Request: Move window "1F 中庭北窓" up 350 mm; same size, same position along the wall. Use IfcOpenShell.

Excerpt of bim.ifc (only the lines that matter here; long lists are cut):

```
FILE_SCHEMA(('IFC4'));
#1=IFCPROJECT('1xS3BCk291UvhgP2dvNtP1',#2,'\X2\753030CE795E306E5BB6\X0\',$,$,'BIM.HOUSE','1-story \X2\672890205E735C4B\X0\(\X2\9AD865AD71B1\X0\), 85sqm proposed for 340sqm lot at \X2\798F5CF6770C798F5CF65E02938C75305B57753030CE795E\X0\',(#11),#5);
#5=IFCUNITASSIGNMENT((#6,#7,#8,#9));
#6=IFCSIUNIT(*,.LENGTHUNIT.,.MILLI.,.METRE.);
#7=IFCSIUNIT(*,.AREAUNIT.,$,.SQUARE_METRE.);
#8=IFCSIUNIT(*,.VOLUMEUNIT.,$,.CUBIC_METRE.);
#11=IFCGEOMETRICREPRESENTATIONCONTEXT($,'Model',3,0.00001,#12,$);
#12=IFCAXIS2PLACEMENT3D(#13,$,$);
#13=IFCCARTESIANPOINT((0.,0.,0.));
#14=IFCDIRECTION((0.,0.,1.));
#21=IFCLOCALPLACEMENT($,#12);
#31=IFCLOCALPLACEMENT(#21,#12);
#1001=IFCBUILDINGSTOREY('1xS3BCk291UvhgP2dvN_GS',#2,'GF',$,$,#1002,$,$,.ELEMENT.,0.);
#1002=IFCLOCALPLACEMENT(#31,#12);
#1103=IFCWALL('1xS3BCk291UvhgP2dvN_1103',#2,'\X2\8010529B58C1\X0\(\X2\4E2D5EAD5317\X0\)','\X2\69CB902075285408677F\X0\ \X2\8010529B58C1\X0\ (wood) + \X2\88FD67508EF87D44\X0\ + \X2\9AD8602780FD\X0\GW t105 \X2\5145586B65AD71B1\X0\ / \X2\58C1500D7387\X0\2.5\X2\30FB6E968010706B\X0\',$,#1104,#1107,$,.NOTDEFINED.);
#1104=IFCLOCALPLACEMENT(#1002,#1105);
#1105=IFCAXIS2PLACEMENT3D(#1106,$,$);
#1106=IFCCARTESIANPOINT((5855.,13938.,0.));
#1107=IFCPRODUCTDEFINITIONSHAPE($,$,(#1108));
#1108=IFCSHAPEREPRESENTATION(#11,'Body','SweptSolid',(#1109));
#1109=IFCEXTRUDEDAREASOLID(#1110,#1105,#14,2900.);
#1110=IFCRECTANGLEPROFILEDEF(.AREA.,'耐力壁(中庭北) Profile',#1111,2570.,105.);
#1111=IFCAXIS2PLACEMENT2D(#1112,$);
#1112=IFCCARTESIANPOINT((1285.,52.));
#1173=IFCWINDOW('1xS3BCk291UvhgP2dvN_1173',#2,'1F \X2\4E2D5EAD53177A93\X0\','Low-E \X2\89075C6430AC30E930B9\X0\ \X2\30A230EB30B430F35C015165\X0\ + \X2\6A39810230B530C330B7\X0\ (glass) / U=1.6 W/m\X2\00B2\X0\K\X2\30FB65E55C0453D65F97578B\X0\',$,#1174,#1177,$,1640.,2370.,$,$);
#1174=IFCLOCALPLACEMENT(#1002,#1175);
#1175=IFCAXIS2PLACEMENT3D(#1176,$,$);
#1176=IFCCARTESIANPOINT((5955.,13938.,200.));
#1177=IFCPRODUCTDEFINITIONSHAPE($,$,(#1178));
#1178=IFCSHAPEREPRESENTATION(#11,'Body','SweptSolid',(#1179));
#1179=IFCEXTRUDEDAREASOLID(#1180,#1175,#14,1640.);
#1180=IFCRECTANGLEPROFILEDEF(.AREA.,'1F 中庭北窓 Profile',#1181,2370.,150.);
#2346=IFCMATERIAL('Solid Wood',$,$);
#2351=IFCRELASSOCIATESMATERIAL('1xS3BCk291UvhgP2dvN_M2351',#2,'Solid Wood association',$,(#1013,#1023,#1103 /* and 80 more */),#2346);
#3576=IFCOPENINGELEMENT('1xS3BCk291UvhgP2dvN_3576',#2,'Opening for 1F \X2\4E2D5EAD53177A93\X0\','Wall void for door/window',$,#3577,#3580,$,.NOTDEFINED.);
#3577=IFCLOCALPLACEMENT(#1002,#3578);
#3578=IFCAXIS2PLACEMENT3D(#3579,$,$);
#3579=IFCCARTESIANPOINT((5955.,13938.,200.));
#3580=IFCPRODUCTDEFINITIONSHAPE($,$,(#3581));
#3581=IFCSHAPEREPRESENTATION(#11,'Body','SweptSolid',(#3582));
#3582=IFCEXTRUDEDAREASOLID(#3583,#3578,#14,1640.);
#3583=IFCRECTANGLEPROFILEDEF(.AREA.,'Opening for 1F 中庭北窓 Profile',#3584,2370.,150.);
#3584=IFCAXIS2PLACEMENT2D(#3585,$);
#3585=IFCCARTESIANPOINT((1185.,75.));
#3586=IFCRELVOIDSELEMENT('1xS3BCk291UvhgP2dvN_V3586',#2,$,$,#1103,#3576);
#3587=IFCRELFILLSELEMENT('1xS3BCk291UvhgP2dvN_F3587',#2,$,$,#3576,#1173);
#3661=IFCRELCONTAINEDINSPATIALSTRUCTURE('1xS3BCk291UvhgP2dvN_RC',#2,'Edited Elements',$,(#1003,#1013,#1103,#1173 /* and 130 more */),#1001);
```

```python
import numpy as np
import ifcopenshell
import ifcopenshell.api.geometry
import ifcopenshell.util.placement
import ifcopenshell.util.unit

model = ifcopenshell.open("bim.ifc")
unit_scale = ifcopenshell.util.unit.calculate_unit_scale(model)

window = model.by_guid("1xS3BCk291UvhgP2dvN_1173")
opening = window.FillsVoids[0].RelatingOpeningElement
dz = 0.35 / unit_scale

shift = np.array([0.0, 0.0, dz])
# The window is not placed relative to its opening, so move both.
for product in (opening, window):
    matrix = ifcopenshell.util.placement.get_local_placement(product.ObjectPlacement)
    matrix[:3, 3] += shift
    ifcopenshell.api.geometry.edit_object_placement(model, product=product, matrix=matrix, is_si=False)

print(f"moved by {dz * unit_scale:+.3f} m")

model.write("bim-out.ifc")
```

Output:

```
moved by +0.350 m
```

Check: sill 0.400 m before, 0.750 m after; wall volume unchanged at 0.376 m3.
